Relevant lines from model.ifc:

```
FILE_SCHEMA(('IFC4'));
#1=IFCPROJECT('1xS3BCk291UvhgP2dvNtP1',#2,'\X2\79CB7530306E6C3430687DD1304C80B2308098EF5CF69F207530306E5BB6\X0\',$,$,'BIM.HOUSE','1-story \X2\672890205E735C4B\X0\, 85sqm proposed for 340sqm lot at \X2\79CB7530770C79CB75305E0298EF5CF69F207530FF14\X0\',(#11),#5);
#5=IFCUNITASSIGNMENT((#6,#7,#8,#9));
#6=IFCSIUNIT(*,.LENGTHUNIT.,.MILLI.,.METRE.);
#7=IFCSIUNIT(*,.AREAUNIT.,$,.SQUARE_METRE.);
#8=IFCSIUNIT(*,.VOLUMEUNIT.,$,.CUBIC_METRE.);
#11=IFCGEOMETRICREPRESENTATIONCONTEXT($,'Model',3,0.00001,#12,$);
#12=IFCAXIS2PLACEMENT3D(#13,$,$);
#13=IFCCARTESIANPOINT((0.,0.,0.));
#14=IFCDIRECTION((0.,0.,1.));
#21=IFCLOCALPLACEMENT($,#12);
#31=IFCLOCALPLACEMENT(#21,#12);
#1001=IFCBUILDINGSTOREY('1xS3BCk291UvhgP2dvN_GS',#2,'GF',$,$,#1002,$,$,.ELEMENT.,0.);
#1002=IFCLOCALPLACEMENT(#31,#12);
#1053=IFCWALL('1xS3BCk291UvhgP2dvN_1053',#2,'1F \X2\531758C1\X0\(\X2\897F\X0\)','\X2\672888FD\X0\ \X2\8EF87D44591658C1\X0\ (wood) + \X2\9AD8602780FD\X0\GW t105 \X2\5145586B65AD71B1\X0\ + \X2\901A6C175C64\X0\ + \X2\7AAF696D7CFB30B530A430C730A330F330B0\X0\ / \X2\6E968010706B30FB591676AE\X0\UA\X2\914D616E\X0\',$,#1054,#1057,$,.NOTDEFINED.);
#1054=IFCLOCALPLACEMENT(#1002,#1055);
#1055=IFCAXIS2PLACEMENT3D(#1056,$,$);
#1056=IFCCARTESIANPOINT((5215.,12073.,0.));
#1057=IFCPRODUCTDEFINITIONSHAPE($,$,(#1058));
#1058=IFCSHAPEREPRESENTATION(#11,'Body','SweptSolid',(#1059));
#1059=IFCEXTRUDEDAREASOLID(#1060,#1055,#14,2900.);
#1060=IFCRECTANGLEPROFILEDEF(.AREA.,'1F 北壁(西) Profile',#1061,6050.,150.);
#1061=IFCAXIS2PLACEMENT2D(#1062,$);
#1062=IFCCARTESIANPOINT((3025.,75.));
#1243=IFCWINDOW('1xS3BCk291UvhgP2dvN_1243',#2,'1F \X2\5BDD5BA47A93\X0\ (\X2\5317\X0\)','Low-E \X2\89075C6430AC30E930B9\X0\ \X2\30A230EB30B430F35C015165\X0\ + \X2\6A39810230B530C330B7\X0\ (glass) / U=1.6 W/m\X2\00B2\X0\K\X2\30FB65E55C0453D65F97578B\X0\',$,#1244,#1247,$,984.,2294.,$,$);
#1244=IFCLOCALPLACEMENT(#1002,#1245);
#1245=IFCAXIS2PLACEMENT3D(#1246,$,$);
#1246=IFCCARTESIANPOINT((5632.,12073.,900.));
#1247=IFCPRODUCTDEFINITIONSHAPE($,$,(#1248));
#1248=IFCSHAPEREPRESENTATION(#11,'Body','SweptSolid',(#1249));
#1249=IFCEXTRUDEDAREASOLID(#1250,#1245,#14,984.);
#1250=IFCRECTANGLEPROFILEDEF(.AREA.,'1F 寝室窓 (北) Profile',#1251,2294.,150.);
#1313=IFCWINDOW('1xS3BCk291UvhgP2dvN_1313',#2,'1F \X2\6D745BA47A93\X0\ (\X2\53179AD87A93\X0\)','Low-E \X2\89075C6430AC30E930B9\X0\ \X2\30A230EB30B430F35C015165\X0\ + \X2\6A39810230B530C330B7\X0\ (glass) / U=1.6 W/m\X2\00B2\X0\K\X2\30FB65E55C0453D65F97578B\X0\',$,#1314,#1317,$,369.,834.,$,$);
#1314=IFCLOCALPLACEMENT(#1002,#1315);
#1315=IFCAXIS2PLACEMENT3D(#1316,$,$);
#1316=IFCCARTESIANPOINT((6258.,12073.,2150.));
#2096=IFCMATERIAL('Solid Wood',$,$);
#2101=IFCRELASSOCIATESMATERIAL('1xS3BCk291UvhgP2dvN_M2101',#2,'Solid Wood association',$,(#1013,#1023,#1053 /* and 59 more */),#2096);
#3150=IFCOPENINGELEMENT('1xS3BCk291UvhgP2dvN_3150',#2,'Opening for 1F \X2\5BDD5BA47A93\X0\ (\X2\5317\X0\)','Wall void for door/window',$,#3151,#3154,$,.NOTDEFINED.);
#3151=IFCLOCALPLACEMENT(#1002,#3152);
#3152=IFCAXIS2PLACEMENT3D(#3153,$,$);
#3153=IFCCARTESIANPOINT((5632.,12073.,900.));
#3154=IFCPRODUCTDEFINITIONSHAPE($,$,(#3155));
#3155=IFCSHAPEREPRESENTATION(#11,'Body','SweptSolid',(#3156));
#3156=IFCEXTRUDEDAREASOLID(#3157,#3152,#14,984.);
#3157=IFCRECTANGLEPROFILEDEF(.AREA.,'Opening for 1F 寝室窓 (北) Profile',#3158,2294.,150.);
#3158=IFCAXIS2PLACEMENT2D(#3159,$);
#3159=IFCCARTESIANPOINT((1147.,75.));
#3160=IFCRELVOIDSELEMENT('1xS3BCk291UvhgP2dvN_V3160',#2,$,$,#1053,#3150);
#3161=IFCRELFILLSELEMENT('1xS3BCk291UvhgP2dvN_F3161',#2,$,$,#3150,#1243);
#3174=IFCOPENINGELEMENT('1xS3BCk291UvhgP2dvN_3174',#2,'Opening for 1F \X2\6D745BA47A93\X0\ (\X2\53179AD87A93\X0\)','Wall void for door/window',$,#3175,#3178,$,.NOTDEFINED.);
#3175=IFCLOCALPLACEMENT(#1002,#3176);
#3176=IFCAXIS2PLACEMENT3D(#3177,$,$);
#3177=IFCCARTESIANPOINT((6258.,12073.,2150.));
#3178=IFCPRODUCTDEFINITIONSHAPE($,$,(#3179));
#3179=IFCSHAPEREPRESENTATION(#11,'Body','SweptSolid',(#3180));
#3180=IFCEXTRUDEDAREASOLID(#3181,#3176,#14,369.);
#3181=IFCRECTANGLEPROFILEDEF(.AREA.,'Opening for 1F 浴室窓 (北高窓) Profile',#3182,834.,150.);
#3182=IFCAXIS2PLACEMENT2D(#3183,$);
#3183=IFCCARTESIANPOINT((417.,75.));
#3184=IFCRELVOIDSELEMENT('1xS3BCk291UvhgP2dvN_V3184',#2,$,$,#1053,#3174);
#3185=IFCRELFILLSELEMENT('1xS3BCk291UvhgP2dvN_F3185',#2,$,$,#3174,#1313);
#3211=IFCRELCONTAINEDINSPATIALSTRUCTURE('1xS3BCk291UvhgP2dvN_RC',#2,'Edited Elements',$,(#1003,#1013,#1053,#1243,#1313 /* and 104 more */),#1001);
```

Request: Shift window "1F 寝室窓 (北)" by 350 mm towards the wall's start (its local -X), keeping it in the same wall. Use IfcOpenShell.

```python
import ifcopenshell
import ifcopenshell.api.geometry
import ifcopenshell.util.placement

model = ifcopenshell.open("model.ifc")

window = model.by_guid("1xS3BCk291UvhgP2dvN_1243")
opening = window.FillsVoids[0].RelatingOpeningElement
wall = opening.VoidsElements[0].RelatingBuildingElement

wall_matrix = ifcopenshell.util.placement.get_local_placement(wall.ObjectPlacement)
shift = wall_matrix[:3, 0] * -350.0
before = ifcopenshell.util.placement.get_local_placement(window.ObjectPlacement)[:3, 3].copy()

# The window is not placed relative to its opening, so move both.
for product in (opening, window):
    matrix = ifcopenshell.util.placement.get_local_placement(product.ObjectPlacement)
    matrix[:3, 3] += shift
    ifcopenshell.api.geometry.edit_object_placement(model, product=product, matrix=matrix, is_si=False)

after = ifcopenshell.util.placement.get_local_placement(window.ObjectPlacement)[:3, 3]
print("window moved by", (after - before).round(3) + 0.0)

model.write("model_edited.ifc")
```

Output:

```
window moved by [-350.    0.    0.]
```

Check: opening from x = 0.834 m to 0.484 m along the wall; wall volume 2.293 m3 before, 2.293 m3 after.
